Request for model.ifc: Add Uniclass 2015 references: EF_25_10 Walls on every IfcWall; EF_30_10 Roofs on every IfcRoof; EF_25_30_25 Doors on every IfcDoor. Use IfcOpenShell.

First a look at what the model holds.

```python
import ifcopenshell

model = ifcopenshell.open("model.ifc")
print(model.schema)
print("classifications:", [c.Name for c in model.by_type("IfcClassification")])
for ifc_class in ("IfcDoor", "IfcRoof", "IfcStair", "IfcWall", "IfcWindow"):
    print(ifc_class, len(model.by_type(ifc_class)))
```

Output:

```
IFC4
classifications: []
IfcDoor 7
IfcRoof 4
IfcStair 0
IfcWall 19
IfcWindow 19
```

```python
import ifcopenshell
import ifcopenshell.api.classification

model = ifcopenshell.open("model.ifc")

system = ifcopenshell.api.classification.add_classification(model, classification="Uniclass 2015")

codes = {
    "IfcWall": ("EF_25_10", "Walls"),
    "IfcRoof": ("EF_30_10", "Roofs"),
    "IfcDoor": ("EF_25_30_25", "Doors"),
}
for ifc_class, (code, name) in codes.items():
    products = model.by_type(ifc_class)
    ifcopenshell.api.classification.add_reference(
        model, products=products, classification=system, identification=code, name=name
    )
    print(code, len(products))

model.write("model_rev.ifc")
```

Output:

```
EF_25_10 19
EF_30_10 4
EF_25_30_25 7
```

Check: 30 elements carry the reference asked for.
